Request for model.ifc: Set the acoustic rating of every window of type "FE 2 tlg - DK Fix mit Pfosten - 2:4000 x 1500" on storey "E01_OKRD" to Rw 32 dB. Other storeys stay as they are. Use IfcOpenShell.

First a look at what the model holds.

```python
import ifcopenshell
import ifcopenshell.util.element

model = ifcopenshell.open("model.ifc")
print(model.schema)
storey = next(s for s in model.by_type("IfcBuildingStorey") if s.Name == "E01_OKRD")
windows = [e for e in ifcopenshell.util.element.get_decomposition(storey) if e.is_a("IfcWindow")]
seen = {}
for e in windows:
    element_type = ifcopenshell.util.element.get_type(e)
    key = (element_type.Name if element_type != e and element_type else None, ifcopenshell.util.element.get_pset(e, "Pset_WindowCommon", "AcousticRating"))
    seen[key] = seen.get(key, 0) + 1
for (name, value), count in sorted(seen.items(), key=str):
    print(count, "x", name, "|", value)
```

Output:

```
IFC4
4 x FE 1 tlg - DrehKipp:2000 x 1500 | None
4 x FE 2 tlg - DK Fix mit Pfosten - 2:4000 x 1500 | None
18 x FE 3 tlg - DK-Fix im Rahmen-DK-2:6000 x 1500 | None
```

```python
import ifcopenshell
import ifcopenshell.api.pset
import ifcopenshell.util.element

model = ifcopenshell.open("model.ifc")

storey = next(s for s in model.by_type("IfcBuildingStorey") if s.Name == "E01_OKRD")
windows = [e for e in ifcopenshell.util.element.get_decomposition(storey) if e.is_a("IfcWindow")]

count = 0
for e in windows:
    element_type = ifcopenshell.util.element.get_type(e)
    if element_type in (None, e) or element_type.Name != "FE 2 tlg - DK Fix mit Pfosten - 2:4000 x 1500":
        continue
    # add_pset returns the element's existing set when there is one.
    pset = ifcopenshell.api.pset.add_pset(model, product=e, name="Pset_WindowCommon")
    ifcopenshell.api.pset.edit_pset(model, pset=pset, properties={"AcousticRating": "Rw 32 dB"})
    count += 1

print(count, "windows updated")

model.write("model_v2.ifc")
```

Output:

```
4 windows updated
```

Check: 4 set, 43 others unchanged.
